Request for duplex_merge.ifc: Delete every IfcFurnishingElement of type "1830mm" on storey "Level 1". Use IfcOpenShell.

First a look at what the model holds.

```python
import ifcopenshell
import ifcopenshell.util.element

model = ifcopenshell.open("duplex_merge.ifc")
print(model.schema)
storey = next(s for s in model.by_type("IfcBuildingStorey") if s.Name == "Level 1")
furniture = [e for e in ifcopenshell.util.element.get_decomposition(storey) if e.is_a("IfcFurnishingElement")]
seen = {}
for e in furniture:
    element_type = ifcopenshell.util.element.get_type(e)
    name = element_type.Name if element_type not in (None, e) else None
    seen[name] = seen.get(name, 0) + 1
for name, count in sorted(seen.items(), key=str):
    print(count, "x", name)
```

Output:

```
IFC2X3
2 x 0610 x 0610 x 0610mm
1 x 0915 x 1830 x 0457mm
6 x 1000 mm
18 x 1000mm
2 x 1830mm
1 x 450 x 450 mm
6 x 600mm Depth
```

```python
import ifcopenshell
import ifcopenshell.api.root
import ifcopenshell.util.element

model = ifcopenshell.open("duplex_merge.ifc")

storey = next(s for s in model.by_type("IfcBuildingStorey") if s.Name == "Level 1")
furniture = [e for e in ifcopenshell.util.element.get_decomposition(storey) if e.is_a("IfcFurnishingElement")]
targets = [e for e in furniture if (t := ifcopenshell.util.element.get_type(e)) not in (None, e) and t.Name == "1830mm"]

for e in targets:
    ifcopenshell.api.root.remove_product(model, product=e)
print(len(targets), "removed")

model.write("duplex_merge_edited.ifc")
```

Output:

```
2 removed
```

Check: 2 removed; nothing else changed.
